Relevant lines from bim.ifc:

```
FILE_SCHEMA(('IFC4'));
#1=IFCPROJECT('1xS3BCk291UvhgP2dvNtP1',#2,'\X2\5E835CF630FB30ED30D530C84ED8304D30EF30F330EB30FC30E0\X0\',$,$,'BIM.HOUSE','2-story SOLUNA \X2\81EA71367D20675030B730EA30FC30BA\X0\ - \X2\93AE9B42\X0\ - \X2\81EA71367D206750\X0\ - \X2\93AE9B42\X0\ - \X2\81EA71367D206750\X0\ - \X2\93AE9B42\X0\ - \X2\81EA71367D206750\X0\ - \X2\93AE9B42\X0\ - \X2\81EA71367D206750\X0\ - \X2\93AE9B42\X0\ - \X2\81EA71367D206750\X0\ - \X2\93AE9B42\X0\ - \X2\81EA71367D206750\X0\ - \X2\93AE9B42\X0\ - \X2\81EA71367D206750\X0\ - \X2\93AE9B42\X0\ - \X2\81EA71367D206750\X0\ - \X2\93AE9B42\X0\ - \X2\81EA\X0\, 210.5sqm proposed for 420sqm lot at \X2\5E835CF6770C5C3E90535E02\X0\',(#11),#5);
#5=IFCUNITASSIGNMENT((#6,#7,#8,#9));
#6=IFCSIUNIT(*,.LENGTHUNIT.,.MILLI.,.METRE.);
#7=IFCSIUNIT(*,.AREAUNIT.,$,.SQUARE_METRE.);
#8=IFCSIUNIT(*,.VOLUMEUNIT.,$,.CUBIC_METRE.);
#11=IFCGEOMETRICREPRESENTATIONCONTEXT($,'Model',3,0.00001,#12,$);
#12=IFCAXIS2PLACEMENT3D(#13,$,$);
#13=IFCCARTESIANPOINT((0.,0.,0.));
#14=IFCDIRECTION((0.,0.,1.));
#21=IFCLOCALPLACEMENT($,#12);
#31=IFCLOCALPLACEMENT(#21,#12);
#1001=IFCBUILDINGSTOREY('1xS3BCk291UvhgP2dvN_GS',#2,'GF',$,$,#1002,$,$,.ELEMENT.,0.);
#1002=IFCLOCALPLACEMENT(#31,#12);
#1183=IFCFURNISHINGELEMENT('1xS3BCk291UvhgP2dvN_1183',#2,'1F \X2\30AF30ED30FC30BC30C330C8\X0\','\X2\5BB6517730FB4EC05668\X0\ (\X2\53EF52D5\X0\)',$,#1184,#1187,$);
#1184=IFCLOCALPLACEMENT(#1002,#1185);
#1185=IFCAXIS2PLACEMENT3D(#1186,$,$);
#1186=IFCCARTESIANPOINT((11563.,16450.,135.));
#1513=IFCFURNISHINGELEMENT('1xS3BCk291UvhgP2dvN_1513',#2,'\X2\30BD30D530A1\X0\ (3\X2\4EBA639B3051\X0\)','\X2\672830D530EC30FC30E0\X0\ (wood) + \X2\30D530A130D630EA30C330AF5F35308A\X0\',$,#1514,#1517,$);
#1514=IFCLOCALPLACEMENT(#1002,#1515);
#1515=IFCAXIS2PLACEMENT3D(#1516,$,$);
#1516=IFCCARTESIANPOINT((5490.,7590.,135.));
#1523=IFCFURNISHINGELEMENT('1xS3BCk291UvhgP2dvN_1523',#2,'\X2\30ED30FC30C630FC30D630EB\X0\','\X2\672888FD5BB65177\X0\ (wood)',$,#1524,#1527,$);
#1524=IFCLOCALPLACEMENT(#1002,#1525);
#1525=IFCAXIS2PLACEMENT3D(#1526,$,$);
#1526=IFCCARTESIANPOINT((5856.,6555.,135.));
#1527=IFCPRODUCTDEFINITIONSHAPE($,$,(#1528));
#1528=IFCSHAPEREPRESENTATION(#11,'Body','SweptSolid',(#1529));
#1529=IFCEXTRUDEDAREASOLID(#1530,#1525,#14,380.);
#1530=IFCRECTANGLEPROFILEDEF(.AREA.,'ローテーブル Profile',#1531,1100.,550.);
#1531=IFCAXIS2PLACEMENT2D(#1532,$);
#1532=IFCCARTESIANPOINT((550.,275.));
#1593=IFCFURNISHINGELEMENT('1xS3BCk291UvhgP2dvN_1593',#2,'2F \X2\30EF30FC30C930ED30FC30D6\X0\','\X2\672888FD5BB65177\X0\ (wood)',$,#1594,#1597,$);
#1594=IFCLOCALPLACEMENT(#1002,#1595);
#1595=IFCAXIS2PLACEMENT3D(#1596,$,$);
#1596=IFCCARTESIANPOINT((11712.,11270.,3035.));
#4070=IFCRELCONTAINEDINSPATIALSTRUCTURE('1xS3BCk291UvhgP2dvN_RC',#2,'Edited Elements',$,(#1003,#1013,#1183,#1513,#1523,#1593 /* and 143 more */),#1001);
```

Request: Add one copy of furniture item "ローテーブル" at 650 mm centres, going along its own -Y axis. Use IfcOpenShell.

```python
import ifcopenshell
import ifcopenshell.api.geometry
import ifcopenshell.api.root
import ifcopenshell.util.element
import ifcopenshell.util.placement
import ifcopenshell.util.unit

model = ifcopenshell.open("bim.ifc")
unit_scale = ifcopenshell.util.unit.calculate_unit_scale(model)


def reuse_history(source, copy):
    """copy_class also copies each property set's owner history, people and application; keep the originals."""
    for rel in copy.IsDefinedBy:
        if rel.is_a("IfcRelDefinesByProperties") and (history := rel.RelatingPropertyDefinition.OwnerHistory):
            rel.RelatingPropertyDefinition.OwnerHistory = source.OwnerHistory
            ifcopenshell.util.element.remove_deep2(model, history)


source = model.by_guid("1xS3BCk291UvhgP2dvN_1523")
base = ifcopenshell.util.placement.get_local_placement(source.ObjectPlacement)
step = -base[:3, 1] * 0.65 / unit_scale

for i in range(1, 2):
    copy = ifcopenshell.api.root.copy_class(model, product=source)
    copy.Representation = ifcopenshell.util.element.copy_deep(
        model, source.Representation, exclude=["IfcGeometricRepresentationContext", "IfcRepresentationMap"]
    )
    reuse_history(source, copy)
    matrix = base.copy()
    matrix[:3, 3] += i * step
    print("added at", matrix[:3, 3].round(3) + 0.0)
    ifcopenshell.api.geometry.edit_object_placement(model, product=copy, matrix=matrix, is_si=False)

model.write("bim_v2.ifc")
```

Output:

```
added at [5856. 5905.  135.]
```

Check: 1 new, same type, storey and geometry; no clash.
